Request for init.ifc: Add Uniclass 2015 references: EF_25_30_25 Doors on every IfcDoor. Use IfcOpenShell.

First a look at what the model holds.

```python
import ifcopenshell

model = ifcopenshell.open("init.ifc")
print(model.schema)
print("classifications:", [c.Name for c in model.by_type("IfcClassification")])
for ifc_class in ("IfcDoor", "IfcRoof", "IfcStair", "IfcWall", "IfcWindow"):
    print(ifc_class, len(model.by_type(ifc_class)))
```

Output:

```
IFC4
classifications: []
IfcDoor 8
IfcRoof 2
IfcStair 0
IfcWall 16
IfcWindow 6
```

```python
import ifcopenshell
import ifcopenshell.api.classification

model = ifcopenshell.open("init.ifc")

system = ifcopenshell.api.classification.add_classification(model, classification="Uniclass 2015")

codes = {
    "IfcDoor": ("EF_25_30_25", "Doors"),
}
for ifc_class, (code, name) in codes.items():
    products = model.by_type(ifc_class)
    ifcopenshell.api.classification.add_reference(
        model, products=products, classification=system, identification=code, name=name
    )
    print(code, len(products))

model.write("init-out.ifc")
```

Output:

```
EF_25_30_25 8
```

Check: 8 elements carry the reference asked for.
